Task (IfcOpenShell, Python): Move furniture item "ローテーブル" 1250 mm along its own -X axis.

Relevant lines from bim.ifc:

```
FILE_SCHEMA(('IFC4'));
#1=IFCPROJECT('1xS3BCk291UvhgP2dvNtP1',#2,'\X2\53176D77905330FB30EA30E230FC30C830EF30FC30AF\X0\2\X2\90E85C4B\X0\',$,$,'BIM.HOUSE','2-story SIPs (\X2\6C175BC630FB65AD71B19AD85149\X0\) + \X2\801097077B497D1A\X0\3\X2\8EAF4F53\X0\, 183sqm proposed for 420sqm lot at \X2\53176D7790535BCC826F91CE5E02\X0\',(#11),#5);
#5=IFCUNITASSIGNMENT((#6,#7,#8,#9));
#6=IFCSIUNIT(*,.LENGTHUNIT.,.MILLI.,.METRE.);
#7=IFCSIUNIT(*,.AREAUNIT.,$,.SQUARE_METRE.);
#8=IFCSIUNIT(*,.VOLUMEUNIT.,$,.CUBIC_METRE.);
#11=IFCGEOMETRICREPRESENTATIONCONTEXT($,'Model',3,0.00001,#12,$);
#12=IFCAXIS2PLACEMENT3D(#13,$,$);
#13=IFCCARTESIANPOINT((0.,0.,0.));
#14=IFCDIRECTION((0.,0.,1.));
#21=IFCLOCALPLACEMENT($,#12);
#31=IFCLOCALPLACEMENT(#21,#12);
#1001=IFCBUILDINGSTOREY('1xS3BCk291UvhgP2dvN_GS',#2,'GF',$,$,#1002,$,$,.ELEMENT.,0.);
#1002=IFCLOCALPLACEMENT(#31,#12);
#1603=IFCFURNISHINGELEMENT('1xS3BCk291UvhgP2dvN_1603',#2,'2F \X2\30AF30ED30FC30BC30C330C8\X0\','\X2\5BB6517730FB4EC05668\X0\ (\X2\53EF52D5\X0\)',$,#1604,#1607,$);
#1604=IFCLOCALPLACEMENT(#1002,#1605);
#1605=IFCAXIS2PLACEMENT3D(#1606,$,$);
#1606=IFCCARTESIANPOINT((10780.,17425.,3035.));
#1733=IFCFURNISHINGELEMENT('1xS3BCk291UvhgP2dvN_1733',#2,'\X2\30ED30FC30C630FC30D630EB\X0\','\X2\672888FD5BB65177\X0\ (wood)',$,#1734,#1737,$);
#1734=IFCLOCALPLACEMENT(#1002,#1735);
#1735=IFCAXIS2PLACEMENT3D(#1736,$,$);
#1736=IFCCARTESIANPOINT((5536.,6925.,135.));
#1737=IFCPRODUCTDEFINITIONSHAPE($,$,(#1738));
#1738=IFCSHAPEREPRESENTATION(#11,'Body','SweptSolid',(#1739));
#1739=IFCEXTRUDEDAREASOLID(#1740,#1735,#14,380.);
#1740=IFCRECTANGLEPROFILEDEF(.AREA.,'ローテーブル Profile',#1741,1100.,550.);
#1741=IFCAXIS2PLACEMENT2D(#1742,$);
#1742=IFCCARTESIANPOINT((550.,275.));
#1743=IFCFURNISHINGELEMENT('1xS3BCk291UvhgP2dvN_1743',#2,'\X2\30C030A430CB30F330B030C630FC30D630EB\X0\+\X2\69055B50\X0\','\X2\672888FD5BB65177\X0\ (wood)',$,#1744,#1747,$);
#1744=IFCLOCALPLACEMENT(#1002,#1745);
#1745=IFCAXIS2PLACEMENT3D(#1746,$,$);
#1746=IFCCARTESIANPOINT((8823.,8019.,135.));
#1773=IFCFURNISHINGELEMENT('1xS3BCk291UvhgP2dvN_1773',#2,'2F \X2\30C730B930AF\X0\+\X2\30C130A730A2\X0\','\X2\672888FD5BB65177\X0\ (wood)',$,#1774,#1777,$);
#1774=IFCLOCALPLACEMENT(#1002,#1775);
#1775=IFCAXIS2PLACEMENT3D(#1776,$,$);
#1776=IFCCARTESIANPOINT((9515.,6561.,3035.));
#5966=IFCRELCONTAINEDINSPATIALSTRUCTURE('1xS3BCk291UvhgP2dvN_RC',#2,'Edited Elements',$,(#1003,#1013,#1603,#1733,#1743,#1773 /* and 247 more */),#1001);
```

```python
import ifcopenshell
import ifcopenshell.api.geometry
import ifcopenshell.util.placement

model = ifcopenshell.open("bim.ifc")

item = model.by_guid("1xS3BCk291UvhgP2dvN_1733")
matrix = ifcopenshell.util.placement.get_local_placement(item.ObjectPlacement)
matrix[:3, 3] -= matrix[:3, 0] * 1250.0
ifcopenshell.api.geometry.edit_object_placement(model, product=item, matrix=matrix, is_si=False)

print(ifcopenshell.util.placement.get_local_placement(item.ObjectPlacement).round(3) + 0.0)

model.write("bim-out.ifc")
```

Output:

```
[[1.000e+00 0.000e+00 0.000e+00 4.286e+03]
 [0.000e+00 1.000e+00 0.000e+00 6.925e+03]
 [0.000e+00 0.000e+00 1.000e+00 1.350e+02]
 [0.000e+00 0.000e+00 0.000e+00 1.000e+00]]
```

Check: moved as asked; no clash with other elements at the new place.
